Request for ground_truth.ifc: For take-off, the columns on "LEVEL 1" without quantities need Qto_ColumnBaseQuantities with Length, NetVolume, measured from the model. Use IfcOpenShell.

First a look at what the model holds.

```python
import ifcopenshell
import ifcopenshell.util.element
import ifcopenshell.util.unit

model = ifcopenshell.open("ground_truth.ifc")
print(model.schema)
for unit_type in ("LENGTHUNIT", "AREAUNIT", "VOLUMEUNIT"):
    print(unit_type, ifcopenshell.util.unit.calculate_unit_scale(model, unit_type))
storey = next(s for s in model.by_type("IfcBuildingStorey") if s.Name == "LEVEL 1")
columns = [e for e in ifcopenshell.util.element.get_decomposition(storey) if e.is_a("IfcColumn")]
for e in sorted(columns, key=lambda e: e.id()):
    print(e.id(), e.is_a(), e.Name, list(ifcopenshell.util.element.get_psets(e, qtos_only=True)), sep=" | ")
```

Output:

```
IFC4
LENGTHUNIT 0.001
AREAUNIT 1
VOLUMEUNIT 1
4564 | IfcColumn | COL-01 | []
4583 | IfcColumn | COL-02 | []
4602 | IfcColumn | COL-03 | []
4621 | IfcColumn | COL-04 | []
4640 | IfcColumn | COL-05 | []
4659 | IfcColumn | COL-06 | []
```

```python
import ifcopenshell
import ifcopenshell.api.pset
import ifcopenshell.geom
import ifcopenshell.util.element
import ifcopenshell.util.shape
import ifcopenshell.util.unit

model = ifcopenshell.open("ground_truth.ifc")
unit_scale = ifcopenshell.util.unit.calculate_unit_scale(model)
volume_scale = ifcopenshell.util.unit.calculate_unit_scale(model, "VOLUMEUNIT")
settings = ifcopenshell.geom.settings()

storey = next(s for s in model.by_type("IfcBuildingStorey") if s.Name == "LEVEL 1")
columns = [e for e in ifcopenshell.util.element.get_decomposition(storey) if e.is_a("IfcColumn")]

for e in sorted(columns, key=lambda e: e.id()):
    if ifcopenshell.util.element.get_psets(e, qtos_only=True, should_inherit=False):
        continue
    # Geometry comes back in metres, in the element's own axes.
    shape = ifcopenshell.geom.create_shape(settings, e)
    values = {
        "Length": ifcopenshell.util.shape.get_z(shape.geometry) / unit_scale,
        "NetVolume": ifcopenshell.util.shape.get_volume(shape.geometry) / volume_scale,
    }
    qto = ifcopenshell.api.pset.add_qto(model, product=e, name="Qto_ColumnBaseQuantities")
    ifcopenshell.api.pset.edit_qto(model, qto=qto, properties=values)
    print(e.id(), {k: round(v, 3) for k, v in values.items()})

model.write("ground_truth_updated.ifc")
```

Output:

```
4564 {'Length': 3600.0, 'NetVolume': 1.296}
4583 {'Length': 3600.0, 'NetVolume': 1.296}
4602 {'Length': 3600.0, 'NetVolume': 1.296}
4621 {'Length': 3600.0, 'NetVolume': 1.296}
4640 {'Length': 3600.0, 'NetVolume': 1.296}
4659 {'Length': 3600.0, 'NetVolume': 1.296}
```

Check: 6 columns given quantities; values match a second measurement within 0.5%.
